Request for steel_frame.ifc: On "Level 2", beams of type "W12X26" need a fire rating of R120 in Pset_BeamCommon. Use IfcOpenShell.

First a look at what the model holds.

```python
import ifcopenshell
import ifcopenshell.util.element

model = ifcopenshell.open("steel_frame.ifc")
print(model.schema)
storey = next(s for s in model.by_type("IfcBuildingStorey") if s.Name == "Level 2")
beams = [e for e in ifcopenshell.util.element.get_decomposition(storey) if e.is_a("IfcBeam")]
seen = {}
for e in beams:
    element_type = ifcopenshell.util.element.get_type(e)
    key = (element_type.Name if element_type != e and element_type else None, ifcopenshell.util.element.get_pset(e, "Pset_BeamCommon", "FireRating"))
    seen[key] = seen.get(key, 0) + 1
for (name, value), count in sorted(seen.items(), key=str):
    print(count, "x", name, "|", value)
```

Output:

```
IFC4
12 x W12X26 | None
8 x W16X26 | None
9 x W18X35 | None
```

```python
import ifcopenshell
import ifcopenshell.api.pset
import ifcopenshell.util.element

model = ifcopenshell.open("steel_frame.ifc")

storey = next(s for s in model.by_type("IfcBuildingStorey") if s.Name == "Level 2")
beams = [e for e in ifcopenshell.util.element.get_decomposition(storey) if e.is_a("IfcBeam")]

count = 0
for e in beams:
    element_type = ifcopenshell.util.element.get_type(e)
    if element_type in (None, e) or element_type.Name != "W12X26":
        continue
    # add_pset returns the element's existing set when there is one.
    pset = ifcopenshell.api.pset.add_pset(model, product=e, name="Pset_BeamCommon")
    ifcopenshell.api.pset.edit_pset(model, pset=pset, properties={"FireRating": "R120"})
    count += 1

print(count, "beams updated")

model.write("steel_frame_edited.ifc")
```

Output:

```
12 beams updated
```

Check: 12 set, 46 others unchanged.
